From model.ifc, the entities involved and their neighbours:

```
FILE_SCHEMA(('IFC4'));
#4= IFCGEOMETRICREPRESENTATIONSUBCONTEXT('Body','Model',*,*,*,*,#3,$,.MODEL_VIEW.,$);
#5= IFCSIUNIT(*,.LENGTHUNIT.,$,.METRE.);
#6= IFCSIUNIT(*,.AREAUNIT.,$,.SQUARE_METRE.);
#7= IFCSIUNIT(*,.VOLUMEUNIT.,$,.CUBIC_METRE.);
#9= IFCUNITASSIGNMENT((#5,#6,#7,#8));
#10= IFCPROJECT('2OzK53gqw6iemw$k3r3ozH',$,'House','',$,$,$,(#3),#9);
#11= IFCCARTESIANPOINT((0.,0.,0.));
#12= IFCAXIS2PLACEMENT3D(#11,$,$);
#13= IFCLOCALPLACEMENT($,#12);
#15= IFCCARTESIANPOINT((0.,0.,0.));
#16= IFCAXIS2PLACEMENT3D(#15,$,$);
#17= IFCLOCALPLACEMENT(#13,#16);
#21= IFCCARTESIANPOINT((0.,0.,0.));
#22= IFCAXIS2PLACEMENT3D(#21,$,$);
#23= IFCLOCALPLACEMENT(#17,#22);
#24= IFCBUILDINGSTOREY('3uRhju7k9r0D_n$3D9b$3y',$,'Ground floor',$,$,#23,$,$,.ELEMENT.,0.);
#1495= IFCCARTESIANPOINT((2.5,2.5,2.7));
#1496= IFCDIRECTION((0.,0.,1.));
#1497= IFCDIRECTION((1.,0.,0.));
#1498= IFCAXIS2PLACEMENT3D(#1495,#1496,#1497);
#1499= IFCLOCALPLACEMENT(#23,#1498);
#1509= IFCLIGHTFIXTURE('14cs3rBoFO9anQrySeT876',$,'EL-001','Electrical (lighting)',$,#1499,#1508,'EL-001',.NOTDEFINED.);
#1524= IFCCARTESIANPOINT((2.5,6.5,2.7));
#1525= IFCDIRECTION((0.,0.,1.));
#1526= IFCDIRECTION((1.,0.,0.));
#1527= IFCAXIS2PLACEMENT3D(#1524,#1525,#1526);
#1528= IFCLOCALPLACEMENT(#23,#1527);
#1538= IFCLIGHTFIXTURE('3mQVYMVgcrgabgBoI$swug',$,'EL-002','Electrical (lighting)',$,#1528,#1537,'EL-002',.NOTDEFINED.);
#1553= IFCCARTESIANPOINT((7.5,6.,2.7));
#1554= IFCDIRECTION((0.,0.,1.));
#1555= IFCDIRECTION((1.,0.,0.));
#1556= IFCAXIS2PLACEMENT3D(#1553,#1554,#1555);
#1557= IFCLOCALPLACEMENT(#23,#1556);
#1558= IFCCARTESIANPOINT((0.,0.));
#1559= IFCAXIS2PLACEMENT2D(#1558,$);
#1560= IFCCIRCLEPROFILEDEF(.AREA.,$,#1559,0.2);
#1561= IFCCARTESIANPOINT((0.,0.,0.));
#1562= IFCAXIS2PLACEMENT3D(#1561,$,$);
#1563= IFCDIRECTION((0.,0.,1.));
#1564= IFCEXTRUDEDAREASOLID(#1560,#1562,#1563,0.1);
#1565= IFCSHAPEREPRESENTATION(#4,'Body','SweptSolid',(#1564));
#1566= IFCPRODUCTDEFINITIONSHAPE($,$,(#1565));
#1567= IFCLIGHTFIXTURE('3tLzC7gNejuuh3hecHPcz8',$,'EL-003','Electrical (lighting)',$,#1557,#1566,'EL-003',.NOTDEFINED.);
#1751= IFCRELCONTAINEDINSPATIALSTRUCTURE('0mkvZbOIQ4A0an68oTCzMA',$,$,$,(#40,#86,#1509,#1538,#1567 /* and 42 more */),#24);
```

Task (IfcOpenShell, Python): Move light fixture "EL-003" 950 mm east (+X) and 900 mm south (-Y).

```python
import ifcopenshell
import ifcopenshell.api.geometry
import ifcopenshell.util.placement
import ifcopenshell.util.unit

model = ifcopenshell.open("model.ifc")
unit_scale = ifcopenshell.util.unit.calculate_unit_scale(model)

item = model.by_guid("3tLzC7gNejuuh3hecHPcz8")
matrix = ifcopenshell.util.placement.get_local_placement(item.ObjectPlacement)
matrix[0, 3] += 0.95 / unit_scale
matrix[1, 3] -= 0.9 / unit_scale
ifcopenshell.api.geometry.edit_object_placement(model, product=item, matrix=matrix, is_si=False)

print(ifcopenshell.util.placement.get_local_placement(item.ObjectPlacement).round(3) + 0.0)

model.write("model-out.ifc")
```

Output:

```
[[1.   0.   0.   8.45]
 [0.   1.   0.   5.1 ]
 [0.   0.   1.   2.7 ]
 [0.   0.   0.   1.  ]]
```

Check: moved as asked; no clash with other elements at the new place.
